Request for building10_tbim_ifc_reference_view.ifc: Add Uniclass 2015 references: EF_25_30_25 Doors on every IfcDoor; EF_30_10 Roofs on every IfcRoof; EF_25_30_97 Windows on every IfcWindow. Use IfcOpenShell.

First a look at what the model holds.

```python
import ifcopenshell

model = ifcopenshell.open("building10_tbim_ifc_reference_view.ifc")
print(model.schema)
print("classifications:", [c.Name for c in model.by_type("IfcClassification")])
for ifc_class in ("IfcDoor", "IfcRoof", "IfcStair", "IfcWall", "IfcWindow"):
    print(ifc_class, len(model.by_type(ifc_class)))
```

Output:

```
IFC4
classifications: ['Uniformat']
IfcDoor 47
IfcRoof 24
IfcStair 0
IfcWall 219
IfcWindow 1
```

```python
import ifcopenshell
import ifcopenshell.api.classification

model = ifcopenshell.open("building10_tbim_ifc_reference_view.ifc")

system = ifcopenshell.api.classification.add_classification(model, classification="Uniclass 2015")

codes = {
    "IfcDoor": ("EF_25_30_25", "Doors"),
    "IfcRoof": ("EF_30_10", "Roofs"),
    "IfcWindow": ("EF_25_30_97", "Windows"),
}
for ifc_class, (code, name) in codes.items():
    products = model.by_type(ifc_class)
    ifcopenshell.api.classification.add_reference(
        model, products=products, classification=system, identification=code, name=name
    )
    print(code, len(products))

model.write("building10_tbim_ifc_reference_view_edited.ifc")
```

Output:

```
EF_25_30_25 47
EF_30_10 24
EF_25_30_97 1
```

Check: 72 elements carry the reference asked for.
